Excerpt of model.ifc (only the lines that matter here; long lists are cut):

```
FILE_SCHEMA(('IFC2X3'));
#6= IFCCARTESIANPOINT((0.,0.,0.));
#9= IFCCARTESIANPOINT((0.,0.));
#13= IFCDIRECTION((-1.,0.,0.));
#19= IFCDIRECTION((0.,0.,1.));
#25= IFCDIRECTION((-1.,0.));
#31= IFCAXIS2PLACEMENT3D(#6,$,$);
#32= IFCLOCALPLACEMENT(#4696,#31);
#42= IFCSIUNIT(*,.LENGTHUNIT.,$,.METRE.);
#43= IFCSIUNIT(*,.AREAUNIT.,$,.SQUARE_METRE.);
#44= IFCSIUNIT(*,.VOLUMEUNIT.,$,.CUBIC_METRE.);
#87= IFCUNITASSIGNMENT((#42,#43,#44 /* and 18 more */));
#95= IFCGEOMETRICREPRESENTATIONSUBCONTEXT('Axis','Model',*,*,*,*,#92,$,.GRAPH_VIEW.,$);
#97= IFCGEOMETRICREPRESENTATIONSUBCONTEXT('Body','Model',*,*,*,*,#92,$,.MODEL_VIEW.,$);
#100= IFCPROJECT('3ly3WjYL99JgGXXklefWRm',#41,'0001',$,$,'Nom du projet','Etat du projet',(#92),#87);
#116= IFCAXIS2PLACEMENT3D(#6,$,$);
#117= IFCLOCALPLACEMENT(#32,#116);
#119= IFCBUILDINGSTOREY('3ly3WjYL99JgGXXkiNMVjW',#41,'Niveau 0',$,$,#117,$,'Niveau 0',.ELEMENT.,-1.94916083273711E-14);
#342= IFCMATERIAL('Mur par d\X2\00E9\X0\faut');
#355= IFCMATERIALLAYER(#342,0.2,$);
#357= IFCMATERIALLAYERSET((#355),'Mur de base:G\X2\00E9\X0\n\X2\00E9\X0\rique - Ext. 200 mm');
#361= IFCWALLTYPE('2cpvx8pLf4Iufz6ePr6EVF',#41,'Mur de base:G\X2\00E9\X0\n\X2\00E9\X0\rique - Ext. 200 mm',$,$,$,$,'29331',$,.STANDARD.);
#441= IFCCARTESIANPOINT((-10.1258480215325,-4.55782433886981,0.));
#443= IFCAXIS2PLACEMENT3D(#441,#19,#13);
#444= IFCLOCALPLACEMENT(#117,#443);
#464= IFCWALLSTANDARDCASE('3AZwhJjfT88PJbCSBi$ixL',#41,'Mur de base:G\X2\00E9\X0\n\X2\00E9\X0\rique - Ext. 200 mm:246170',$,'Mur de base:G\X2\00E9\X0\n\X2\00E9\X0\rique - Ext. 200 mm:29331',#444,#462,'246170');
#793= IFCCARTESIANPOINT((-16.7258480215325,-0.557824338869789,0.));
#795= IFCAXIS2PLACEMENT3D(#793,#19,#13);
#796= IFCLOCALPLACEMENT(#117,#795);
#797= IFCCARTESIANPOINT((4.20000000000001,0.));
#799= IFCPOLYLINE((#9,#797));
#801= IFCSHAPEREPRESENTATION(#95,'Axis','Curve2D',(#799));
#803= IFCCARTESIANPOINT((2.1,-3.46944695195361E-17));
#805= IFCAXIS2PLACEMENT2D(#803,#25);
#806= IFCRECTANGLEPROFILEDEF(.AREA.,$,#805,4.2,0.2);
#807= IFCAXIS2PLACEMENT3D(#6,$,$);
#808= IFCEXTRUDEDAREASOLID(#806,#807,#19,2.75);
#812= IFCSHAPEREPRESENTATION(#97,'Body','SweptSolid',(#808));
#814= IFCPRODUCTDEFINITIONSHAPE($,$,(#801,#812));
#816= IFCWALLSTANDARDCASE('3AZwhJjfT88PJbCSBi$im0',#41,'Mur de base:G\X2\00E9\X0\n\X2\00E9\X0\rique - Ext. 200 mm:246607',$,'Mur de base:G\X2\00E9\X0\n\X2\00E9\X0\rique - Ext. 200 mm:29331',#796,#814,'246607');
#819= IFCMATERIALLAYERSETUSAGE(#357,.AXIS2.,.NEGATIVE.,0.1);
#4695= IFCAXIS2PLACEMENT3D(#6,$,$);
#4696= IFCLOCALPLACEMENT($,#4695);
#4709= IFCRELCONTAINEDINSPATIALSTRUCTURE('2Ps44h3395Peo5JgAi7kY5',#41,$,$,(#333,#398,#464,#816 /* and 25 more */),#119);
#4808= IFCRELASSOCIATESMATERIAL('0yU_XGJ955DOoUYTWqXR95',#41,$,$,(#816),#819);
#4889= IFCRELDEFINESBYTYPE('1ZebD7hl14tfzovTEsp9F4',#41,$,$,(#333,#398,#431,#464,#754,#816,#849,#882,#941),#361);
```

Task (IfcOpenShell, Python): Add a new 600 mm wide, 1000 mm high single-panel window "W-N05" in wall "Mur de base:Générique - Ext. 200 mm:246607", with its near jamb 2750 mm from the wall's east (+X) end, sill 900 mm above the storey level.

```python
import numpy as np
import ifcopenshell
import ifcopenshell.api.feature
import ifcopenshell.api.geometry
import ifcopenshell.api.root
import ifcopenshell.api.spatial
import ifcopenshell.api.type
import ifcopenshell.geom
import ifcopenshell.util.element
import ifcopenshell.util.placement
import ifcopenshell.util.representation
import ifcopenshell.util.shape
import ifcopenshell.util.unit

model = ifcopenshell.open("model.ifc")
unit_scale = ifcopenshell.util.unit.calculate_unit_scale(model)
settings = ifcopenshell.geom.settings()


def volume(element):
    """Net volume in cubic metres, openings subtracted."""
    shape = ifcopenshell.geom.create_shape(settings, element)
    return ifcopenshell.util.shape.get_volume(shape.geometry)


wall = model.by_guid("3AZwhJjfT88PJbCSBi$im0")
storey = ifcopenshell.util.element.get_container(wall, ifc_class="IfcBuildingStorey")
context = ifcopenshell.util.representation.get_context(model, "Model", "Body", "MODEL_VIEW")
before = volume(wall)

width, height, from_end, sill = 0.6, 1, 2.75, 0.9  # metres

# The wall runs along its own X axis, and the end named is its -X end.
wall_shape = ifcopenshell.geom.create_shape(settings, wall)
x, y, z = ifcopenshell.util.shape.get_vertices(wall_shape.geometry).T
start = x.min() + from_end
face, thickness = float(y.min()), float(y.max() - y.min())
wall_matrix = ifcopenshell.util.placement.get_local_placement(wall.ObjectPlacement)
level = ifcopenshell.util.placement.get_local_placement(storey.ObjectPlacement)[2, 3]


def in_wall(x, y):
    """Placement at x, y metres in the wall's axes, at sill height."""
    matrix = wall_matrix.copy()
    matrix[:, 3] = wall_matrix @ np.array([x / unit_scale, y / unit_scale, 0.0, 1.0])
    matrix[2, 3] = level + sill / unit_scale
    return matrix


# Opening: a box that overshoots both wall faces by 50 mm.
opening = ifcopenshell.api.root.create_entity(model, ifc_class="IfcOpeningElement")
box = ifcopenshell.api.geometry.add_wall_representation(
    model, context=context, length=width, height=height, thickness=thickness + 0.1
)
ifcopenshell.api.geometry.assign_representation(model, product=opening, representation=box)
ifcopenshell.api.geometry.edit_object_placement(model, product=opening, matrix=in_wall(start, face - 0.05), is_si=False)
ifcopenshell.api.feature.add_feature(model, feature=opening, element=wall)

window = ifcopenshell.api.root.create_entity(model, ifc_class="IfcWindow", name="W-N05")
window.OverallWidth, window.OverallHeight = width / unit_scale, height / unit_scale
body = ifcopenshell.api.geometry.add_window_representation(
    model,
    context=context,
    overall_width=window.OverallWidth,
    overall_height=window.OverallHeight,
    partition_type="SINGLE_PANEL",
)
ifcopenshell.api.geometry.assign_representation(model, product=window, representation=body)
ifcopenshell.api.spatial.assign_container(model, products=[window], relating_structure=storey)
fills = ifcopenshell.api.feature.add_filling(model, opening=opening, element=window)
fills.OwnerHistory = window.OwnerHistory  # required in IFC2X3

# IFC2X3 keeps the operation on the window style.
style = ifcopenshell.api.root.create_entity(model, ifc_class="IfcWindowStyle", name="W-N05")
style.OperationType, style.ConstructionType = "SINGLE_PANEL", "NOTDEFINED"
style.ParameterTakesPrecedence = style.Sizeable = False
ifcopenshell.api.type.assign_type(model, related_objects=[window], relating_type=style)

# Centre the window in the wall's thickness.
ifcopenshell.api.geometry.edit_object_placement(model, product=window, matrix=in_wall(start, face), is_si=False)
window_shape = ifcopenshell.geom.create_shape(settings, window)
depth = ifcopenshell.util.shape.get_vertices(window_shape.geometry)[:, 1]
offset = face + thickness / 2 - (depth.min() + depth.max()) / 2
ifcopenshell.api.geometry.edit_object_placement(model, product=window, matrix=in_wall(start, offset), is_si=False)

after = volume(wall)

print(f"wall volume {before:.3f} -> {after:.3f} m3")

model.write("model_edited.ifc")
```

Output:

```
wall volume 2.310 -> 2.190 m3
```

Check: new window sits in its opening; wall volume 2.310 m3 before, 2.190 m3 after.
